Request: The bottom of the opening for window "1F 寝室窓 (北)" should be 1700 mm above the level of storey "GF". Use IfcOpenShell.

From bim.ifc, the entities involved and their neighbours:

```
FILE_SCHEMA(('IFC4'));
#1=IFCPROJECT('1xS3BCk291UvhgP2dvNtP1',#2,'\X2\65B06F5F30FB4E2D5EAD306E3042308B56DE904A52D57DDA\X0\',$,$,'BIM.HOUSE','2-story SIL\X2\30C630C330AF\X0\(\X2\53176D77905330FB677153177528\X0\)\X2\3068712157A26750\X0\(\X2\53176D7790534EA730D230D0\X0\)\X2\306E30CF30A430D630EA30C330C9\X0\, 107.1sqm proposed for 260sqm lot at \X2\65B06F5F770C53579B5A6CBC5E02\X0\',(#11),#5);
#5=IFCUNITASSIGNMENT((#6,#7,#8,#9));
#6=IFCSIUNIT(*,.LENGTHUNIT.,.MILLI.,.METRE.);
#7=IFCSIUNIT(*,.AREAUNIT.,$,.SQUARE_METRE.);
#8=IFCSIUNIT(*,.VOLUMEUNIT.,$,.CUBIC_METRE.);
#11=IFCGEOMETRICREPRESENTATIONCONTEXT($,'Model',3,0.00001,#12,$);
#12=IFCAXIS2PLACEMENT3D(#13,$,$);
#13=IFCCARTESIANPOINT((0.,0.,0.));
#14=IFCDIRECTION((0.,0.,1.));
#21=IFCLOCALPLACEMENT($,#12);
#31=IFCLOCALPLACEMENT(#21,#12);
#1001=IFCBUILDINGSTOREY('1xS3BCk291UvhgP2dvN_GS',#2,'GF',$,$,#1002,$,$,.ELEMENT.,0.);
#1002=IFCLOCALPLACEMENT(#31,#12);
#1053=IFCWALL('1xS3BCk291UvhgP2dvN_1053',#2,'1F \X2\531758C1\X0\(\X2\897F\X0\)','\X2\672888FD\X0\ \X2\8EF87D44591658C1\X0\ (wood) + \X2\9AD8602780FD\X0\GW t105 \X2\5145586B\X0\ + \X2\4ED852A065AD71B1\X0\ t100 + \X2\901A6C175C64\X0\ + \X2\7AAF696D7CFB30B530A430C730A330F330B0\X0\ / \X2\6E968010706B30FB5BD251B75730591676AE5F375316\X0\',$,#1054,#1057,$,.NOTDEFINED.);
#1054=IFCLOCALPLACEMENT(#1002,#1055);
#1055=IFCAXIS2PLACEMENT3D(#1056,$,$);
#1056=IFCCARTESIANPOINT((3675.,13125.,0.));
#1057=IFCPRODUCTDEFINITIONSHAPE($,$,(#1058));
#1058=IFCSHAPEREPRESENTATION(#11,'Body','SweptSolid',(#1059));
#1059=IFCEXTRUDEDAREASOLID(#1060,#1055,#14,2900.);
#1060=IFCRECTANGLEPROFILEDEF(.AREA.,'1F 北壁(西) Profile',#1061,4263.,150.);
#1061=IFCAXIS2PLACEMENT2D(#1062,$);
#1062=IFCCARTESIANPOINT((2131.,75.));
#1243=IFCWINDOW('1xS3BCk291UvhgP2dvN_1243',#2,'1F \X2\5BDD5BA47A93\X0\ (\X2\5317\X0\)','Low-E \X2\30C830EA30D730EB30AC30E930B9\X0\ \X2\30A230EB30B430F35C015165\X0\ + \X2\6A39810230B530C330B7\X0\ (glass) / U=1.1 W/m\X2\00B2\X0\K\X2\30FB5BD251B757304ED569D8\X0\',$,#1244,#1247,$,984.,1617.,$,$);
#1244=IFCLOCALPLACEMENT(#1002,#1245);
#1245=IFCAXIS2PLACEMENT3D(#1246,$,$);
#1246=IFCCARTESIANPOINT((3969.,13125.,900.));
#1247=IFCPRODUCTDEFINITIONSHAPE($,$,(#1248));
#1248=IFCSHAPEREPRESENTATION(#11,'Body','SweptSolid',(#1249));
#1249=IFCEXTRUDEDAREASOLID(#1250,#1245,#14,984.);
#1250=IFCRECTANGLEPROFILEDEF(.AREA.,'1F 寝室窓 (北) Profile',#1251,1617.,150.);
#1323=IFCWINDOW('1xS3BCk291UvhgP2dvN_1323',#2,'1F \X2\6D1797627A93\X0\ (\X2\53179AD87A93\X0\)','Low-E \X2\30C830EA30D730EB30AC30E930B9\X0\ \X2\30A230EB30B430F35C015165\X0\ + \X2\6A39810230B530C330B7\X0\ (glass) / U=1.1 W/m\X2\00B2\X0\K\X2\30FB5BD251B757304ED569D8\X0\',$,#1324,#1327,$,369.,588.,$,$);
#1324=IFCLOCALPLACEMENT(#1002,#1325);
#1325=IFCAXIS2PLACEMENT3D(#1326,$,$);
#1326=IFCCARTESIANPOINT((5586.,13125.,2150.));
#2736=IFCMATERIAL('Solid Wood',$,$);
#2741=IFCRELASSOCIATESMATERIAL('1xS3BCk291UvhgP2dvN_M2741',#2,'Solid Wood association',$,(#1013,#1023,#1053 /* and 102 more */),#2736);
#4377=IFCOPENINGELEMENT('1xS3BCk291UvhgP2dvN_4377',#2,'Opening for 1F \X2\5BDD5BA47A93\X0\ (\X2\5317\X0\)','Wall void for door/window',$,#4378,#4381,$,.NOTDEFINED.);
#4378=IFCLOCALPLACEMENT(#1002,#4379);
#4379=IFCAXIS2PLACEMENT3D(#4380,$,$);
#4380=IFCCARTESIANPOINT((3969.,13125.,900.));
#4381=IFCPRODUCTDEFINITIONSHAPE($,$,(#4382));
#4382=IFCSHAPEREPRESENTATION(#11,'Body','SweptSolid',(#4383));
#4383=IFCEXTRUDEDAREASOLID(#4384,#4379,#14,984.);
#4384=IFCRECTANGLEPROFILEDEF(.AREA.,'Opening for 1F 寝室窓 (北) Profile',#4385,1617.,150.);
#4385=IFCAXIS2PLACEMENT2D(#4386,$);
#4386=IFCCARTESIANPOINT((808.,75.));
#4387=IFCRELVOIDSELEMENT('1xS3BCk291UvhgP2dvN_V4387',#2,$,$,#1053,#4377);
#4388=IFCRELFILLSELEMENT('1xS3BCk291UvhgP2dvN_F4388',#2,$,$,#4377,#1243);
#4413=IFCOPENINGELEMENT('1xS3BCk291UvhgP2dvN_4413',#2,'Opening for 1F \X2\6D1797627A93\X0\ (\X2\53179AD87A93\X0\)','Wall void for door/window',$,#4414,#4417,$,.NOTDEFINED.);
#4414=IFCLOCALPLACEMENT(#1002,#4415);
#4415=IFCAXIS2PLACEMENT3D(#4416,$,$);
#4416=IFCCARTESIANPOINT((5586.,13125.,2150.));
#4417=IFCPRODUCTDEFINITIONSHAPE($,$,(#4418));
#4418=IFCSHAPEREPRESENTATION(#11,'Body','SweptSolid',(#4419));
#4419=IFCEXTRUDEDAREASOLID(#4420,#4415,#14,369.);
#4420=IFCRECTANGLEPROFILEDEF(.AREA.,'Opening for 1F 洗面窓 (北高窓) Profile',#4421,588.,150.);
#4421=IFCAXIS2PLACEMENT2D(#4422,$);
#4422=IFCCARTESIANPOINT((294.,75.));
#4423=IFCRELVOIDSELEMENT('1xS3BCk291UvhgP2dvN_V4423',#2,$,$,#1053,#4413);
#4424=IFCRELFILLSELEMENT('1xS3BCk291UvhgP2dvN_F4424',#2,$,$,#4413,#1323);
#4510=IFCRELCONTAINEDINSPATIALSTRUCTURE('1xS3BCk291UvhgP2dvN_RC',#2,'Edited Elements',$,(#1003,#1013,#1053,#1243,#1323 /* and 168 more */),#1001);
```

```python
import numpy as np
import ifcopenshell
import ifcopenshell.api.geometry
import ifcopenshell.geom
import ifcopenshell.util.element
import ifcopenshell.util.placement
import ifcopenshell.util.shape
import ifcopenshell.util.unit

model = ifcopenshell.open("bim.ifc")
unit_scale = ifcopenshell.util.unit.calculate_unit_scale(model)

window = model.by_guid("1xS3BCk291UvhgP2dvN_1243")
opening = window.FillsVoids[0].RelatingOpeningElement
storey = ifcopenshell.util.element.get_container(window, ifc_class="IfcBuildingStorey")
level = ifcopenshell.util.placement.get_local_placement(storey.ObjectPlacement)[2, 3]

# The opening's origin need not be at the sill, so measure its lowest point.
shape = ifcopenshell.geom.create_shape(ifcopenshell.geom.settings(), opening)
bottom = ifcopenshell.util.shape.get_shape_bottom_elevation(shape, shape.geometry) / unit_scale
dz = level + 1.7 / unit_scale - bottom

shift = np.array([0.0, 0.0, dz])
# The window is not placed relative to its opening, so move both.
for product in (opening, window):
    matrix = ifcopenshell.util.placement.get_local_placement(product.ObjectPlacement)
    matrix[:3, 3] += shift
    ifcopenshell.api.geometry.edit_object_placement(model, product=product, matrix=matrix, is_si=False)

print(f"moved by {dz * unit_scale:+.3f} m")

model.write("bim_rev.ifc")
```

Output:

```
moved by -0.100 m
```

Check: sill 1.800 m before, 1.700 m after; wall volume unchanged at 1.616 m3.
